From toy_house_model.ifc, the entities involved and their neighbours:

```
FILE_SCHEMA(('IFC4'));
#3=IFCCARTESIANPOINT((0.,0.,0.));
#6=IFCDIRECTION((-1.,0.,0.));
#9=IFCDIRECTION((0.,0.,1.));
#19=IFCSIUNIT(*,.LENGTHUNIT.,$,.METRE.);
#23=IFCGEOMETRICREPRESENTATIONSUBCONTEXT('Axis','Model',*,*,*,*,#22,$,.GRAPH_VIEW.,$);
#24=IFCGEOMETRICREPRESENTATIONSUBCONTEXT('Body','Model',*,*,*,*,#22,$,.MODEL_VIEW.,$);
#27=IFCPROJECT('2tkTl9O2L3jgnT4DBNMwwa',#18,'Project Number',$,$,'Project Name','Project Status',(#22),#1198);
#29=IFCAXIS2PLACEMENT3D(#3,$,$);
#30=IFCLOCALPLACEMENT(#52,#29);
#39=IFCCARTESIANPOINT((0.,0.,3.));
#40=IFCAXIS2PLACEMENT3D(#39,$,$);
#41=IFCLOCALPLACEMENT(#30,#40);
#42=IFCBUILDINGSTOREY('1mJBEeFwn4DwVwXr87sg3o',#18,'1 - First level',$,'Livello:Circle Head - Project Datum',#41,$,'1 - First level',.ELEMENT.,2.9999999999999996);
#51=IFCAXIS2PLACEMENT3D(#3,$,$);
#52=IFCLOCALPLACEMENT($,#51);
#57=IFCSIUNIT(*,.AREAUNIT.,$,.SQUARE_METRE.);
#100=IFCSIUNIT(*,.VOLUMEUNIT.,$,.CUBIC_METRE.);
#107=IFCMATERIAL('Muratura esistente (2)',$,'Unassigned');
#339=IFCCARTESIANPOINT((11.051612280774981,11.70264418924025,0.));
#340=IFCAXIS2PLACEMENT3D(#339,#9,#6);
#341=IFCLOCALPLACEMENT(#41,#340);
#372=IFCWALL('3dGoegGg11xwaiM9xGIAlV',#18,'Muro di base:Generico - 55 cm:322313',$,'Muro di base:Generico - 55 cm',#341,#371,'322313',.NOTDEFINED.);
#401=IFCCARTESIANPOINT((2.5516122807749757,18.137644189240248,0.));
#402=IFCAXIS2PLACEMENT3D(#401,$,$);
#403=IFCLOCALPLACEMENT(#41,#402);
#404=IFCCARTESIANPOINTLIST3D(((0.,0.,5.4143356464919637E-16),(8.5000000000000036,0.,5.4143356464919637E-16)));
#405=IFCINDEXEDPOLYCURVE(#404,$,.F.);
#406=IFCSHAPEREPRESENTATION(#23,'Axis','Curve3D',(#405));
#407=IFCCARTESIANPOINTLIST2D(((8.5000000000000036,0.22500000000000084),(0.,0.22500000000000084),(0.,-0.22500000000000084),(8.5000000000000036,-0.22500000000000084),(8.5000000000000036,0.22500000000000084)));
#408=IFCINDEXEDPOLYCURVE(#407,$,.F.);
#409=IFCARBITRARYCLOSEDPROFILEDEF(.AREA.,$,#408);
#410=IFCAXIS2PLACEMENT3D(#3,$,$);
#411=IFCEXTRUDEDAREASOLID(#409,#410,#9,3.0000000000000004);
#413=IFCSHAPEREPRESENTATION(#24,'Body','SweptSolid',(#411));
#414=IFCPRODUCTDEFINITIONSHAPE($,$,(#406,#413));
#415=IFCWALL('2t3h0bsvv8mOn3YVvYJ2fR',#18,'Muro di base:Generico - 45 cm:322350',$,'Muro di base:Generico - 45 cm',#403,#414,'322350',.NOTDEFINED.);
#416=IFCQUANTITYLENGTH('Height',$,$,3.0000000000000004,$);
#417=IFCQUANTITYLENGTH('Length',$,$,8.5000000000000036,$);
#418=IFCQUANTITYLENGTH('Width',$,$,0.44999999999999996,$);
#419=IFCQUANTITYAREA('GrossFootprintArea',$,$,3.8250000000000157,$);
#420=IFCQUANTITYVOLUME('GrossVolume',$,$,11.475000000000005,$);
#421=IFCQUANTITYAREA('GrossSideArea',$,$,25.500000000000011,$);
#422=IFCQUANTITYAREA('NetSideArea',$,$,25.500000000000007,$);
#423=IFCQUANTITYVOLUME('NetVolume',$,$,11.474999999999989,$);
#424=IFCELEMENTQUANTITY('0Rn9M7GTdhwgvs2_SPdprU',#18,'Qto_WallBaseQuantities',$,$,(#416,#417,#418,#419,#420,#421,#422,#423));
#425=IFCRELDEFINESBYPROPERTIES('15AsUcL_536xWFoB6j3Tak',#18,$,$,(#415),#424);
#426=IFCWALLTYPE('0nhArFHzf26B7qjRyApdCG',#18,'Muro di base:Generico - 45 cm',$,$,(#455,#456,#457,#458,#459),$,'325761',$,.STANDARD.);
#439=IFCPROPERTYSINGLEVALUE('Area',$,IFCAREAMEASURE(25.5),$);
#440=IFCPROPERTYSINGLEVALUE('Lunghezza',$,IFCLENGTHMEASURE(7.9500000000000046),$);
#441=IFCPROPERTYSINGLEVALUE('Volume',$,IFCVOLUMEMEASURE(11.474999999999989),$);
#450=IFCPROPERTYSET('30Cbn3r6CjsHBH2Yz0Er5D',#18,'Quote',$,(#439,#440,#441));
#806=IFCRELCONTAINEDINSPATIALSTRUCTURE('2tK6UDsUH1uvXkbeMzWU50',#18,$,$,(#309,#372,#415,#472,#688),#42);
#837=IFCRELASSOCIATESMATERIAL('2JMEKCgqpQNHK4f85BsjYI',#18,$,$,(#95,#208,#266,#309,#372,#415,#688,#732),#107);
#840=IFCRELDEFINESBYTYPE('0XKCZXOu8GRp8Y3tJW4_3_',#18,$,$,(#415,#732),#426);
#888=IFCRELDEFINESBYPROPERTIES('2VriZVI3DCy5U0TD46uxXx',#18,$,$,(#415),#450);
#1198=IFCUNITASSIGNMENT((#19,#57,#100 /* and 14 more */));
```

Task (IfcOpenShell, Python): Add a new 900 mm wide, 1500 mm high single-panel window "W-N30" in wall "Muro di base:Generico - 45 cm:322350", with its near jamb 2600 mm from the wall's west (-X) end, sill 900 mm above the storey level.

```python
import numpy as np
import ifcopenshell
import ifcopenshell.api.feature
import ifcopenshell.api.geometry
import ifcopenshell.api.pset
import ifcopenshell.api.root
import ifcopenshell.api.spatial
import ifcopenshell.geom
import ifcopenshell.util.element
import ifcopenshell.util.placement
import ifcopenshell.util.representation
import ifcopenshell.util.shape
import ifcopenshell.util.unit

model = ifcopenshell.open("toy_house_model.ifc")
unit_scale = ifcopenshell.util.unit.calculate_unit_scale(model)
area_scale = ifcopenshell.util.unit.calculate_unit_scale(model, "AREAUNIT")
volume_scale = ifcopenshell.util.unit.calculate_unit_scale(model, "VOLUMEUNIT")
settings = ifcopenshell.geom.settings()


def volume(element):
    """Net volume in cubic metres, openings subtracted."""
    shape = ifcopenshell.geom.create_shape(settings, element)
    return ifcopenshell.util.shape.get_volume(shape.geometry)


wall = model.by_id(415)
storey = ifcopenshell.util.element.get_container(wall, ifc_class="IfcBuildingStorey")
context = ifcopenshell.util.representation.get_context(model, "Model", "Body", "MODEL_VIEW")
before = volume(wall)

width, height, from_end, sill = 0.9, 1.5, 2.6, 0.9  # metres

# The wall runs along its own X axis, and the end named is its -X end.
wall_shape = ifcopenshell.geom.create_shape(settings, wall)
x, y, z = ifcopenshell.util.shape.get_vertices(wall_shape.geometry).T
start = x.min() + from_end
face, thickness = float(y.min()), float(y.max() - y.min())
wall_matrix = ifcopenshell.util.placement.get_local_placement(wall.ObjectPlacement)
level = ifcopenshell.util.placement.get_local_placement(storey.ObjectPlacement)[2, 3]


def in_wall(x, y):
    """Placement at x, y metres in the wall's axes, at sill height."""
    matrix = wall_matrix.copy()
    matrix[:, 3] = wall_matrix @ np.array([x / unit_scale, y / unit_scale, 0.0, 1.0])
    matrix[2, 3] = level + sill / unit_scale
    return matrix


# Opening: a box that overshoots both wall faces by 50 mm.
opening = ifcopenshell.api.root.create_entity(model, ifc_class="IfcOpeningElement", predefined_type="OPENING")
box = ifcopenshell.api.geometry.add_wall_representation(
    model, context=context, length=width, height=height, thickness=thickness + 0.1
)
ifcopenshell.api.geometry.assign_representation(model, product=opening, representation=box)
ifcopenshell.api.geometry.edit_object_placement(model, product=opening, matrix=in_wall(start, face - 0.05), is_si=False)
ifcopenshell.api.feature.add_feature(model, feature=opening, element=wall)

window = ifcopenshell.api.root.create_entity(model, ifc_class="IfcWindow", name="W-N30", predefined_type="WINDOW")
window.OverallWidth, window.OverallHeight = width / unit_scale, height / unit_scale
window.PartitioningType = "SINGLE_PANEL"
body = ifcopenshell.api.geometry.add_window_representation(
    model,
    context=context,
    overall_width=window.OverallWidth,
    overall_height=window.OverallHeight,
    partition_type="SINGLE_PANEL",
)
ifcopenshell.api.geometry.assign_representation(model, product=window, representation=body)
ifcopenshell.api.spatial.assign_container(model, products=[window], relating_structure=storey)
ifcopenshell.api.feature.add_filling(model, opening=opening, element=window)

# Centre the window in the wall's thickness.
ifcopenshell.api.geometry.edit_object_placement(model, product=window, matrix=in_wall(start, face), is_si=False)
window_shape = ifcopenshell.geom.create_shape(settings, window)
depth = ifcopenshell.util.shape.get_vertices(window_shape.geometry)[:, 1]
offset = face + thickness / 2 - (depth.min() + depth.max()) / 2
ifcopenshell.api.geometry.edit_object_placement(model, product=window, matrix=in_wall(start, offset), is_si=False)

after = volume(wall)

# Update the wall's stored quantities.
qto = model.by_id(ifcopenshell.util.element.get_pset(wall, "Qto_WallBaseQuantities", should_inherit=False)["id"])
ifcopenshell.api.pset.edit_qto(model, qto=qto, properties={
    "NetSideArea": after / thickness / area_scale,
    "NetVolume": after / volume_scale,
})
pset = model.by_id(ifcopenshell.util.element.get_pset(wall, "Quote", should_inherit=False)["id"])
ifcopenshell.api.pset.edit_pset(model, pset=pset, properties={
    "Area": model.create_entity("IfcAreaMeasure", after / thickness / area_scale),
    "Volume": model.create_entity("IfcVolumeMeasure", after / volume_scale),
})

print(f"wall volume {before:.3f} -> {after:.3f} m3")

model.write("toy_house_model_v2.ifc")
```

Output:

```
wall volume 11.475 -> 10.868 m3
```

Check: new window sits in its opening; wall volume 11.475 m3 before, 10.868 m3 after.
